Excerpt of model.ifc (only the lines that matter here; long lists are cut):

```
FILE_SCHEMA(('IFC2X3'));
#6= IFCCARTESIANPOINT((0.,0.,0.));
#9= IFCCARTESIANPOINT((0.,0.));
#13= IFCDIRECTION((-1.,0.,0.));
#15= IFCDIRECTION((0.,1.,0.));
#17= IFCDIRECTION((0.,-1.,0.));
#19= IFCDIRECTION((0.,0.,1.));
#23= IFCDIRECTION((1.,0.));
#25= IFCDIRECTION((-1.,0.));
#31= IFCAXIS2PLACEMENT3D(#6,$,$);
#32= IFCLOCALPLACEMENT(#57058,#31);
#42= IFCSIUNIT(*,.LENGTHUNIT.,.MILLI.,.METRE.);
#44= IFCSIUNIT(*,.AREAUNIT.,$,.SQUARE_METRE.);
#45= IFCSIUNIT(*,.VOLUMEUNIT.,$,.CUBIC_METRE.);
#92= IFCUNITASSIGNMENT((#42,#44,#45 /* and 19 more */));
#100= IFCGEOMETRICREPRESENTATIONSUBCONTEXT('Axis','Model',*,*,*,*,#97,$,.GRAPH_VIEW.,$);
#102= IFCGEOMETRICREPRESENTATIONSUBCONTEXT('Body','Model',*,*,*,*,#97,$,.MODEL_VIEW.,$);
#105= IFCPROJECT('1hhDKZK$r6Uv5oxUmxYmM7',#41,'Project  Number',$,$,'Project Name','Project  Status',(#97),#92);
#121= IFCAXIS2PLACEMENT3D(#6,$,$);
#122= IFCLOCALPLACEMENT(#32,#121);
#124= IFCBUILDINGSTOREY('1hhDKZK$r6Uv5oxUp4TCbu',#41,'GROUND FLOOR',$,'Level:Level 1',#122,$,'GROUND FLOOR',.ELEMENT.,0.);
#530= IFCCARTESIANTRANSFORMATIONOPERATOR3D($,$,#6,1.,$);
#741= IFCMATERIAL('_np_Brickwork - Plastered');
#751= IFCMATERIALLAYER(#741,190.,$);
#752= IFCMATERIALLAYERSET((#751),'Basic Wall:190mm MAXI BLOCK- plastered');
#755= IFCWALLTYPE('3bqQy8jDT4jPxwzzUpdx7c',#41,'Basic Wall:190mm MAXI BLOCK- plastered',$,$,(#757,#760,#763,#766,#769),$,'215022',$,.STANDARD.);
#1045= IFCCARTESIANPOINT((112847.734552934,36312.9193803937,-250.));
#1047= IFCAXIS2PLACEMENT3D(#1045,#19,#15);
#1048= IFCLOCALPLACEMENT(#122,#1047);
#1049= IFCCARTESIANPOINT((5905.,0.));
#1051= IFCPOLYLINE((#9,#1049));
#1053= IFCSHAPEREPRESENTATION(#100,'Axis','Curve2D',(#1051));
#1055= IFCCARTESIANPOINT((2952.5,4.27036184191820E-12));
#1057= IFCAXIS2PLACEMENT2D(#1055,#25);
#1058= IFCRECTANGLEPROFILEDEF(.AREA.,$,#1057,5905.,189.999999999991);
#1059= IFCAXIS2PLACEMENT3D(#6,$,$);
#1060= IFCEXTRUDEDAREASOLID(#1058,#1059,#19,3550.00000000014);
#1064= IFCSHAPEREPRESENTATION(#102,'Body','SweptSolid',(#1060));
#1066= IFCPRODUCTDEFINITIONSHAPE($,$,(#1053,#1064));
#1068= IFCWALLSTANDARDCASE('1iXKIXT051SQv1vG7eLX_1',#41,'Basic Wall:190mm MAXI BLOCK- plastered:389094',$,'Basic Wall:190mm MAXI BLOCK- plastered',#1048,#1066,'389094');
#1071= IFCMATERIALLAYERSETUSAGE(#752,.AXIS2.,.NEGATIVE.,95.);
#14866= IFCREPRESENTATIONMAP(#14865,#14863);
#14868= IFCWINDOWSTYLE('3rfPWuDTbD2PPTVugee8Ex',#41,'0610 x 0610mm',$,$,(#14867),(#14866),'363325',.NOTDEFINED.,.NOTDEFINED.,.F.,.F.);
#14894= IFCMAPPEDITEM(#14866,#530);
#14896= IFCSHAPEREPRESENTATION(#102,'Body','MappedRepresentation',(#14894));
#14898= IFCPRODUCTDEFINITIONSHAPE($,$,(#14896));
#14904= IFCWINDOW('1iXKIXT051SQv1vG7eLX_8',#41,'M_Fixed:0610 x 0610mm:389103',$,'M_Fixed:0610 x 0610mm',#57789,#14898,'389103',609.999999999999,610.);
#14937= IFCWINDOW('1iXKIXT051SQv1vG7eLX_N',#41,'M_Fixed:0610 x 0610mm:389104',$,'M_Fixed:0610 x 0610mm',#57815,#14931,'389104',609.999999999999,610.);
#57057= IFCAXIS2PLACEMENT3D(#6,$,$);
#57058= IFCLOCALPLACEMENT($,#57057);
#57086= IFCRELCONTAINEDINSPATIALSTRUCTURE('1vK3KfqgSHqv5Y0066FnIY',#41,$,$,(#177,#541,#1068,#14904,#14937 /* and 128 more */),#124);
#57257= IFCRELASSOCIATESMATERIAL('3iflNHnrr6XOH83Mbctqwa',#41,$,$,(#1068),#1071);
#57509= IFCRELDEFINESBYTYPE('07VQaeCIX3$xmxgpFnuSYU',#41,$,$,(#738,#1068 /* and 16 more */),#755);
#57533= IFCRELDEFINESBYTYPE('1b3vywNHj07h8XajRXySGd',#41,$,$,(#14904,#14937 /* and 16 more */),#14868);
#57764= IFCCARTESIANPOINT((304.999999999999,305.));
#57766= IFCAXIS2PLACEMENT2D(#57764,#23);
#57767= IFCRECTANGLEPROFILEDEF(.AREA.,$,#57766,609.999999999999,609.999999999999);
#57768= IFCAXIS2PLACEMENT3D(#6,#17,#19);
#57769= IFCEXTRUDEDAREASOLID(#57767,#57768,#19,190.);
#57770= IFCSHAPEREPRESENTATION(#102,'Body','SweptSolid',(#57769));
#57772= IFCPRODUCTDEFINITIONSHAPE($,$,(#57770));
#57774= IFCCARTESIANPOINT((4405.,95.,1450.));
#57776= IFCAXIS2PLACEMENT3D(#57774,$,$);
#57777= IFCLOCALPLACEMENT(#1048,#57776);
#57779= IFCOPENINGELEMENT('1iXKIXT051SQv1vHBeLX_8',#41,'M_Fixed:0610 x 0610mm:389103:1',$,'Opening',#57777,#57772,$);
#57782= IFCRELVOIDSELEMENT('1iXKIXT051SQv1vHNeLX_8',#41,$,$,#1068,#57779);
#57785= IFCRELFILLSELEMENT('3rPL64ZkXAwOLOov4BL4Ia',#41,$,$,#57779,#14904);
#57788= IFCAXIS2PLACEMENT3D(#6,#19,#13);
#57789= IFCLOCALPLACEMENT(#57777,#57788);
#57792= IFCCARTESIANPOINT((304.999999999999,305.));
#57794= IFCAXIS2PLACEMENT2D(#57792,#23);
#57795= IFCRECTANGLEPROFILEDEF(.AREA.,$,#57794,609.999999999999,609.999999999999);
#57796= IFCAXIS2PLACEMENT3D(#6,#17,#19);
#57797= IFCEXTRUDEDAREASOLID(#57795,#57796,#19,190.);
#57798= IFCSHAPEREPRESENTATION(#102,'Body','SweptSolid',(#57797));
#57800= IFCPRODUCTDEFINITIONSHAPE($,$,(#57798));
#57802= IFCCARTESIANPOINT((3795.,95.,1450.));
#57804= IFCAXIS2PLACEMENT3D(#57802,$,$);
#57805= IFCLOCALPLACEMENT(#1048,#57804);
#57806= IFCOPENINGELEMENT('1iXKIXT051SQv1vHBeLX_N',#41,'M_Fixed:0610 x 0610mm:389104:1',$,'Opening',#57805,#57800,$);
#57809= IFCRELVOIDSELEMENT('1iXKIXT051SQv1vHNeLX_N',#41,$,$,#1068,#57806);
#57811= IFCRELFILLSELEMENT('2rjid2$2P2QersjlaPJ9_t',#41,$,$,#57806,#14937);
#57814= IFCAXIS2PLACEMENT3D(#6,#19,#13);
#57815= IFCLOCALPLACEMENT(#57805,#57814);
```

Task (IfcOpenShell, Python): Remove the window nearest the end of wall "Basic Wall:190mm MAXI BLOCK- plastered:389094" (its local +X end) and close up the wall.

```python
import ifcopenshell
import ifcopenshell.api.feature
import ifcopenshell.api.root
import ifcopenshell.geom
import ifcopenshell.util.shape

model = ifcopenshell.open("model.ifc")
settings = ifcopenshell.geom.settings()


def volume(element):
    """Net volume in cubic metres, openings subtracted."""
    shape = ifcopenshell.geom.create_shape(settings, element)
    return ifcopenshell.util.shape.get_volume(shape.geometry)


window = model.by_guid("1iXKIXT051SQv1vG7eLX_8")
opening = window.FillsVoids[0].RelatingOpeningElement
wall = opening.VoidsElements[0].RelatingBuildingElement
before = volume(wall)

ifcopenshell.api.root.remove_product(model, product=window)
ifcopenshell.api.feature.remove_feature(model, feature=opening)

after = volume(wall)

print(f"wall volume {before:.3f} -> {after:.3f} m3")

model.write("model_updated.ifc")
```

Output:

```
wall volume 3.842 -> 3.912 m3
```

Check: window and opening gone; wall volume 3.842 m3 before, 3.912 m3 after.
